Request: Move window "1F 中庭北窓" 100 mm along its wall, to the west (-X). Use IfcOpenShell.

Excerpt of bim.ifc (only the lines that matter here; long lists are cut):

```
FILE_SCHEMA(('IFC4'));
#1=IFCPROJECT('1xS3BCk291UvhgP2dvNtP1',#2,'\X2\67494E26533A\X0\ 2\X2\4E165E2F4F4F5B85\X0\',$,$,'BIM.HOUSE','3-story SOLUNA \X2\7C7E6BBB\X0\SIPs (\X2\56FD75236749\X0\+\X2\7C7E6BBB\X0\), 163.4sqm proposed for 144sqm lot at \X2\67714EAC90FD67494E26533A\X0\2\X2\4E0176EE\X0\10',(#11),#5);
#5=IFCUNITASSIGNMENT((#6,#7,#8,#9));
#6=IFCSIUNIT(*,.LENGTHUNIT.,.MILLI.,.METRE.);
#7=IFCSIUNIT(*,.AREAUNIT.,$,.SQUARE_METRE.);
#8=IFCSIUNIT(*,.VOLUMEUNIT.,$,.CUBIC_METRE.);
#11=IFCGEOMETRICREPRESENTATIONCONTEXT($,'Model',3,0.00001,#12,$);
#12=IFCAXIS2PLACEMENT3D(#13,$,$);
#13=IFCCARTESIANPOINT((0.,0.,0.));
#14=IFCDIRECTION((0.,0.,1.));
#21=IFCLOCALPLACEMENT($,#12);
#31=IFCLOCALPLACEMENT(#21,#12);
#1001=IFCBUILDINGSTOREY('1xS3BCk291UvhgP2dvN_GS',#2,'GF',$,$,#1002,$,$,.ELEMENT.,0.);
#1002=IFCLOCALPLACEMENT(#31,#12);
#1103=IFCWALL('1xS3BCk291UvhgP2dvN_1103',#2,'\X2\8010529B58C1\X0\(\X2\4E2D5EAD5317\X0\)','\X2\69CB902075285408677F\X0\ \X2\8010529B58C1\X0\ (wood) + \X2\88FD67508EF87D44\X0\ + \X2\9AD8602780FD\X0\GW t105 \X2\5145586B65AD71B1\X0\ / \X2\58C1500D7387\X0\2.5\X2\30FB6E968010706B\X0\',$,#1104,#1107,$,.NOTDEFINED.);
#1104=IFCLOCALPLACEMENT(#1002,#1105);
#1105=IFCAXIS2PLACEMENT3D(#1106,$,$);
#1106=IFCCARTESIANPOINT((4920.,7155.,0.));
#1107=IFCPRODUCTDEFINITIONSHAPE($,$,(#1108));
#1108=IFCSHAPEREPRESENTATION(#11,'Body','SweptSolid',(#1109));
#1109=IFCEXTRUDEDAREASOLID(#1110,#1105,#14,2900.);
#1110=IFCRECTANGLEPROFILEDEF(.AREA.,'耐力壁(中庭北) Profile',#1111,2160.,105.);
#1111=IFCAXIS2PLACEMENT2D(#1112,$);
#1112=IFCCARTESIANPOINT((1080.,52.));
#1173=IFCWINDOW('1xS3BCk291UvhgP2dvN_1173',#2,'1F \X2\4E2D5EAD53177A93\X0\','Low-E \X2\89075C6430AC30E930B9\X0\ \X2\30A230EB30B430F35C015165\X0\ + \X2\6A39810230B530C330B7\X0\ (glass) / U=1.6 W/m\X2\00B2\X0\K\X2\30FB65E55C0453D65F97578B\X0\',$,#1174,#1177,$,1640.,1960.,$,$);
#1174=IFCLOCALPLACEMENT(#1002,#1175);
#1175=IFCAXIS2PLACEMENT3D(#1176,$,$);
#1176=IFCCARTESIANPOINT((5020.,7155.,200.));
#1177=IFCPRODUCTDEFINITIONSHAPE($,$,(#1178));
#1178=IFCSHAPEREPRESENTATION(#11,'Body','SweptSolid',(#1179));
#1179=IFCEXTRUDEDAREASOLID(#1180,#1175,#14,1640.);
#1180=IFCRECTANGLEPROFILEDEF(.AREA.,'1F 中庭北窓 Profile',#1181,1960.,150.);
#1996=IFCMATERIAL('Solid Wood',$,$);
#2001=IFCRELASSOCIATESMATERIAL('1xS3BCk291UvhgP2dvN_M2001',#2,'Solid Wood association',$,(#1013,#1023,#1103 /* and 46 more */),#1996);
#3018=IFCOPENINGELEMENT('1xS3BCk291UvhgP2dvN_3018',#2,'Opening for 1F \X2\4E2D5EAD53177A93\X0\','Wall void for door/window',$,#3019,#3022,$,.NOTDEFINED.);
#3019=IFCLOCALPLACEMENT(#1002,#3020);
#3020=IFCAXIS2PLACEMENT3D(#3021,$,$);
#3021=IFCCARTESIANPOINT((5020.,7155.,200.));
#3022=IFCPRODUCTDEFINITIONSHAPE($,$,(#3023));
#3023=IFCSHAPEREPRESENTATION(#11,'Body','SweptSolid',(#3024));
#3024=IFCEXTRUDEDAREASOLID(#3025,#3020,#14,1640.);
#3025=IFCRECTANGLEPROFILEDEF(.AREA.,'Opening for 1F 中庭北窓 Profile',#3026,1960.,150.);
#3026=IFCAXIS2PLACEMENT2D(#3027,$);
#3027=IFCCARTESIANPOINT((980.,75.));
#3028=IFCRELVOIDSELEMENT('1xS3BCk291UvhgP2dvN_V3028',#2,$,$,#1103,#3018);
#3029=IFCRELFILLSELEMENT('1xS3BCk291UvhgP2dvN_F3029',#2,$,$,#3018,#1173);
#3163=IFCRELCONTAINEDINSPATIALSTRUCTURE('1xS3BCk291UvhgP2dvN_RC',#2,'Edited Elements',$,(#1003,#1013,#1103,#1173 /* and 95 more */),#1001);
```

```python
import ifcopenshell
import ifcopenshell.api.geometry
import ifcopenshell.util.placement
import ifcopenshell.util.unit

model = ifcopenshell.open("bim.ifc")
unit_scale = ifcopenshell.util.unit.calculate_unit_scale(model)

window = model.by_guid("1xS3BCk291UvhgP2dvN_1173")
opening = window.FillsVoids[0].RelatingOpeningElement
wall = opening.VoidsElements[0].RelatingBuildingElement

wall_matrix = ifcopenshell.util.placement.get_local_placement(wall.ObjectPlacement)
shift = wall_matrix[:3, 0] * -0.1 / unit_scale
before = ifcopenshell.util.placement.get_local_placement(window.ObjectPlacement)[:3, 3].copy()

# The window is not placed relative to its opening, so move both.
for product in (opening, window):
    matrix = ifcopenshell.util.placement.get_local_placement(product.ObjectPlacement)
    matrix[:3, 3] += shift
    ifcopenshell.api.geometry.edit_object_placement(model, product=product, matrix=matrix, is_si=False)

after = ifcopenshell.util.placement.get_local_placement(window.ObjectPlacement)[:3, 3]
print("window moved by", (after - before).round(3) + 0.0)

model.write("bim_edited.ifc")
```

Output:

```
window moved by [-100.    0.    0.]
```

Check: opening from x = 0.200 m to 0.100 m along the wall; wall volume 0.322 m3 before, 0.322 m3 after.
